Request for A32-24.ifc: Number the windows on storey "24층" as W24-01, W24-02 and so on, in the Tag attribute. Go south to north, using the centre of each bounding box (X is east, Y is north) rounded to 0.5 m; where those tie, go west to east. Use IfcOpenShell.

First a look at what the model holds.

```python
import ifcopenshell
import ifcopenshell.util.element
import ifcopenshell.util.placement

model = ifcopenshell.open("A32-24.ifc")
print(model.schema)
storey = next(s for s in model.by_type("IfcBuildingStorey") if s.Name == "24층")
windows = [e for e in ifcopenshell.util.element.get_decomposition(storey) if e.is_a("IfcWindow")]
for e in sorted(windows, key=lambda e: e.id()):
    origin = ifcopenshell.util.placement.get_local_placement(e.ObjectPlacement)[:3, 3]
    print(e.id(), e.Tag, e.Name, origin.round(2) + 0.0, sep=" | ")
```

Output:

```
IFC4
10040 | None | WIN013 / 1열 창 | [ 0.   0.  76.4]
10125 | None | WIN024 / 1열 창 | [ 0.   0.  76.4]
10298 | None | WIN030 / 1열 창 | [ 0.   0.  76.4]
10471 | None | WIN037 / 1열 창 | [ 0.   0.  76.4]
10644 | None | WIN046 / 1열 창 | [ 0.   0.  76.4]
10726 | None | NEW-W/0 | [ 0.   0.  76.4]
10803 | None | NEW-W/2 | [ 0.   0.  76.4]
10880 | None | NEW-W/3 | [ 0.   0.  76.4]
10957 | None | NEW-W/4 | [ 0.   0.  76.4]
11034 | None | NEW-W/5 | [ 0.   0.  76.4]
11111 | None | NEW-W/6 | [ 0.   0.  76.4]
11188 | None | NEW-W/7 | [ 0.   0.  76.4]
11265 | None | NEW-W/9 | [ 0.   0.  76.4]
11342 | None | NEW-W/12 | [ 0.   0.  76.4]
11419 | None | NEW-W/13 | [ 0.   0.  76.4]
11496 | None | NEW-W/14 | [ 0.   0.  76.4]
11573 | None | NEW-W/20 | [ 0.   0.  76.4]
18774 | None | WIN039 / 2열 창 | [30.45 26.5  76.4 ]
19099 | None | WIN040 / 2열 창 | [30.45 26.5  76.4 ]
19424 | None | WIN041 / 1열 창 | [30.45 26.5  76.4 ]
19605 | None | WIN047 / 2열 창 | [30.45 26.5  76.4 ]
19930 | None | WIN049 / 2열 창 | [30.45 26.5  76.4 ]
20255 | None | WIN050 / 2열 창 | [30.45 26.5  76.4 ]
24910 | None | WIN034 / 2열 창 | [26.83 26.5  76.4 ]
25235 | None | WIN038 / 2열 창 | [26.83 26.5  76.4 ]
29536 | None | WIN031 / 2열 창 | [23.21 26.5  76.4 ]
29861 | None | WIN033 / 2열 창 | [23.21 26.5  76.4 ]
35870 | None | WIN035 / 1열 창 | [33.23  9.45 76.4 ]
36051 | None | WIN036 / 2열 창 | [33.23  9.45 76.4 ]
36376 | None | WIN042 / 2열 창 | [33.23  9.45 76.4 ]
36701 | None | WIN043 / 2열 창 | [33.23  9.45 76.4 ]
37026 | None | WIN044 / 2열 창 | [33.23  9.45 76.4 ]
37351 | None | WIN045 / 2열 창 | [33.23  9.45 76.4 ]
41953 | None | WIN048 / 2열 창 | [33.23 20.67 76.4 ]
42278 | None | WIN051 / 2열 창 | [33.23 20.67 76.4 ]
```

```python
import ifcopenshell
import ifcopenshell.geom
import ifcopenshell.util.element
import ifcopenshell.util.shape

model = ifcopenshell.open("A32-24.ifc")
settings = ifcopenshell.geom.settings()
settings.set("use-world-coords", True)


def centre(element):
    shape = ifcopenshell.geom.create_shape(settings, element)
    return ifcopenshell.util.shape.get_bbox_centroid(shape.geometry)


storey = next(s for s in model.by_type("IfcBuildingStorey") if s.Name == "24층")
windows = [e for e in ifcopenshell.util.element.get_decomposition(storey) if e.is_a("IfcWindow")]

# Insertion points can sit at a corner or the storey origin, so sort by the geometry (in metres).
centres = {e: centre(e) for e in windows}
windows.sort(key=lambda e: (round(centres[e][1] / 0.5), centres[e][0]))

for i, e in enumerate(windows, start=1):
    number = f"W24-{i:02d}"
    e.Tag = number
    print(e.id(), number)

model.write("A32-24_rev.ifc")
```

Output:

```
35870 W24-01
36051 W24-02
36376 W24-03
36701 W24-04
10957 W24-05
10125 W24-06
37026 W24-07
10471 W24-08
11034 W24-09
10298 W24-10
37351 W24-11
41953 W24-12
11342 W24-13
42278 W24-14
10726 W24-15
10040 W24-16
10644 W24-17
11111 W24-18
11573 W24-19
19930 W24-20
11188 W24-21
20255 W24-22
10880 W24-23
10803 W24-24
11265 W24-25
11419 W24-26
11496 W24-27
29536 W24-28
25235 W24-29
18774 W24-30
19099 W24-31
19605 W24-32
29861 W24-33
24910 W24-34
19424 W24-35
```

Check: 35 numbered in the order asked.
